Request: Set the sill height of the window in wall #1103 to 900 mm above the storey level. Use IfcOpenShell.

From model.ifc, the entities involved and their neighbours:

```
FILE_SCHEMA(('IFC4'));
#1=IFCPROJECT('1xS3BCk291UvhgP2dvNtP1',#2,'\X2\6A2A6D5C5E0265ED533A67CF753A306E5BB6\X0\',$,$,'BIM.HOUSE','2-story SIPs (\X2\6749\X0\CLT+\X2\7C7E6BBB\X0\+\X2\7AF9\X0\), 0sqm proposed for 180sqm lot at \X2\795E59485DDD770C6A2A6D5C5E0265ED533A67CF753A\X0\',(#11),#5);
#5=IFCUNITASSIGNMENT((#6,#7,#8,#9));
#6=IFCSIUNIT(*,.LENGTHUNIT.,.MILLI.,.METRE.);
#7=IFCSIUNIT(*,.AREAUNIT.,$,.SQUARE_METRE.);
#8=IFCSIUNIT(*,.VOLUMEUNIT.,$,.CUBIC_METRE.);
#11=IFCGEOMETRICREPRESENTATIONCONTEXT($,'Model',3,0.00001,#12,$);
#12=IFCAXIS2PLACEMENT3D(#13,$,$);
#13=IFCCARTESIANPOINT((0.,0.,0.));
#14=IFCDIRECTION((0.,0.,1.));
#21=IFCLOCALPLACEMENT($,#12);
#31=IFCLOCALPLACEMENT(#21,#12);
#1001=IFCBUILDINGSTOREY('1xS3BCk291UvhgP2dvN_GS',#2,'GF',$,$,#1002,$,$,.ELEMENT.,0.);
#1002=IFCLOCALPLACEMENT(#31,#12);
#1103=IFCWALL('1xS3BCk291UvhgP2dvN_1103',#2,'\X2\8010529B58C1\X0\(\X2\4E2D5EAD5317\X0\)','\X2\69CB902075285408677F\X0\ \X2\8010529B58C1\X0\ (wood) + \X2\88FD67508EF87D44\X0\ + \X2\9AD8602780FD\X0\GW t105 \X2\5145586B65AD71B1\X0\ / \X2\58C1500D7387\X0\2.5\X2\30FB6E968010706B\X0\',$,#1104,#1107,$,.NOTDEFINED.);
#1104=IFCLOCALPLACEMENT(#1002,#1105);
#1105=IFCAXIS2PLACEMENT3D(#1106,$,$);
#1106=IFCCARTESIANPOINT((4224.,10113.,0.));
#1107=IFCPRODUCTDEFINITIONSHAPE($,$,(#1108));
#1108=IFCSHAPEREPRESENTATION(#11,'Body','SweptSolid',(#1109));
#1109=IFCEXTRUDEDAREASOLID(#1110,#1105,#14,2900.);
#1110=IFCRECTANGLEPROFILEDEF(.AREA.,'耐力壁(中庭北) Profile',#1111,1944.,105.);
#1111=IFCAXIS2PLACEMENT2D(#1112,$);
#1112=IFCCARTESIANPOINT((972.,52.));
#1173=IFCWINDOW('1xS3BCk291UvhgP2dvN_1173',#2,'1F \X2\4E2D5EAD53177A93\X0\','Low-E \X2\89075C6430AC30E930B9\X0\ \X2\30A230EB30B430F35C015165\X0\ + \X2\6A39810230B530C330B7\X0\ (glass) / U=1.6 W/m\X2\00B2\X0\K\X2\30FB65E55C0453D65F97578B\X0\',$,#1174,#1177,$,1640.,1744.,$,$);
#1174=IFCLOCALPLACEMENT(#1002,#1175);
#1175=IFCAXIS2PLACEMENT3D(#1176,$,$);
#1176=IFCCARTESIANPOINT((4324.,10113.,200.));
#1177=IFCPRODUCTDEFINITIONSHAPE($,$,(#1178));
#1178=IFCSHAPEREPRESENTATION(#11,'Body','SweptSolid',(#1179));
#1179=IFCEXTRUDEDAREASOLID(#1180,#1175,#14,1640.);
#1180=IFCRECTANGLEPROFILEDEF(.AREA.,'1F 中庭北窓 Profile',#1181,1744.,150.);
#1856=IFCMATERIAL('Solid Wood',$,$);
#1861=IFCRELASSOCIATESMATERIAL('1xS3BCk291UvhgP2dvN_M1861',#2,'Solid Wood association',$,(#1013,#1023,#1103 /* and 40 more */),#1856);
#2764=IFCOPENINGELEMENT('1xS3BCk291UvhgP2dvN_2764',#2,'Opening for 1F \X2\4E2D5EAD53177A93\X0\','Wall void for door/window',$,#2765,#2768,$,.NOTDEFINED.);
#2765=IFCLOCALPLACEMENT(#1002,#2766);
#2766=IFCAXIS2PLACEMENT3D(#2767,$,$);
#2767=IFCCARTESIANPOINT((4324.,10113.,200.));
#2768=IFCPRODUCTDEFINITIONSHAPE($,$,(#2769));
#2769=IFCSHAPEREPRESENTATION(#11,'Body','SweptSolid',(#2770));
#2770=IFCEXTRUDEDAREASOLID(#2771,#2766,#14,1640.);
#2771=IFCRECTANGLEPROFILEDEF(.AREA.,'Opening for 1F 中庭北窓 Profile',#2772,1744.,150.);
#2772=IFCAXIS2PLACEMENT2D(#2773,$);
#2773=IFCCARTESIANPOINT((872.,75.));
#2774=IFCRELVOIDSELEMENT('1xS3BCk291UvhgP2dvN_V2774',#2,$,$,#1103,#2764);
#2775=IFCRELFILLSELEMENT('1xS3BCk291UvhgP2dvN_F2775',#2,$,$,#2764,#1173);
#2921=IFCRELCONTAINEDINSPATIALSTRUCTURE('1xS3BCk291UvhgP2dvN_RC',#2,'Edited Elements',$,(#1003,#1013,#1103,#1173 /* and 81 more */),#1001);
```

```python
import numpy as np
import ifcopenshell
import ifcopenshell.api.geometry
import ifcopenshell.geom
import ifcopenshell.util.element
import ifcopenshell.util.placement
import ifcopenshell.util.shape
import ifcopenshell.util.unit

model = ifcopenshell.open("model.ifc")
unit_scale = ifcopenshell.util.unit.calculate_unit_scale(model)

window = model.by_guid("1xS3BCk291UvhgP2dvN_1173")
opening = window.FillsVoids[0].RelatingOpeningElement
storey = ifcopenshell.util.element.get_container(window, ifc_class="IfcBuildingStorey")
level = ifcopenshell.util.placement.get_local_placement(storey.ObjectPlacement)[2, 3]

# The opening's origin need not be at the sill, so measure its lowest point.
shape = ifcopenshell.geom.create_shape(ifcopenshell.geom.settings(), opening)
bottom = ifcopenshell.util.shape.get_shape_bottom_elevation(shape, shape.geometry) / unit_scale
dz = level + 0.9 / unit_scale - bottom

shift = np.array([0.0, 0.0, dz])
# The window is not placed relative to its opening, so move both.
for product in (opening, window):
    matrix = ifcopenshell.util.placement.get_local_placement(product.ObjectPlacement)
    matrix[:3, 3] += shift
    ifcopenshell.api.geometry.edit_object_placement(model, product=product, matrix=matrix, is_si=False)

print(f"moved by {dz * unit_scale:+.3f} m")

model.write("model_rev.ifc")
```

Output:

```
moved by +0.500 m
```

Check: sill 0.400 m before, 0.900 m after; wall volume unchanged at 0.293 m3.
